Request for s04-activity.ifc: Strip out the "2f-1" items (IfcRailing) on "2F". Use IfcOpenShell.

First a look at what the model holds.

```python
import ifcopenshell
import ifcopenshell.util.element

model = ifcopenshell.open("s04-activity.ifc")
print(model.schema)
storey = next(s for s in model.by_type("IfcBuildingStorey") if s.Name == "2F")
railings = [e for e in ifcopenshell.util.element.get_decomposition(storey) if e.is_a("IfcRailing")]
seen = {}
for e in railings:
    element_type = ifcopenshell.util.element.get_type(e)
    name = element_type.Name if element_type not in (None, e) else None
    seen[name] = seen.get(name, 0) + 1
for name, count in sorted(seen.items(), key=str):
    print(count, "x", name)
```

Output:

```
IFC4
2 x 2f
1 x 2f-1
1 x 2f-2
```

```python
import ifcopenshell
import ifcopenshell.api.root
import ifcopenshell.util.element

model = ifcopenshell.open("s04-activity.ifc")

storey = next(s for s in model.by_type("IfcBuildingStorey") if s.Name == "2F")
railings = [e for e in ifcopenshell.util.element.get_decomposition(storey) if e.is_a("IfcRailing")]
targets = [e for e in railings if (t := ifcopenshell.util.element.get_type(e)) not in (None, e) and t.Name == "2f-1"]

for e in targets:
    ifcopenshell.api.root.remove_product(model, product=e)
print(len(targets), "removed")

model.write("s04-activity-out.ifc")
```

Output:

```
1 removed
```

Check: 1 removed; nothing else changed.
